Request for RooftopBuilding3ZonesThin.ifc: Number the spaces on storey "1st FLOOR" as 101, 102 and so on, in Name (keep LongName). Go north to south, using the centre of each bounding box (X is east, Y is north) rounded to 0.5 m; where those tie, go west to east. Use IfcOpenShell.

First a look at what the model holds.

```python
import ifcopenshell
import ifcopenshell.util.element
import ifcopenshell.util.placement

model = ifcopenshell.open("RooftopBuilding3ZonesThin.ifc")
print(model.schema)
storey = next(s for s in model.by_type("IfcBuildingStorey") if s.Name == "1st FLOOR")
spaces = [e for e in ifcopenshell.util.element.get_decomposition(storey) if e.is_a("IfcSpace")]
for e in sorted(spaces, key=lambda e: e.id()):
    origin = ifcopenshell.util.placement.get_local_placement(e.ObjectPlacement)[:3, 3]
    print(e.id(), e.Name, e.LongName, origin.round(2) + 0.0, sep=" | ")
```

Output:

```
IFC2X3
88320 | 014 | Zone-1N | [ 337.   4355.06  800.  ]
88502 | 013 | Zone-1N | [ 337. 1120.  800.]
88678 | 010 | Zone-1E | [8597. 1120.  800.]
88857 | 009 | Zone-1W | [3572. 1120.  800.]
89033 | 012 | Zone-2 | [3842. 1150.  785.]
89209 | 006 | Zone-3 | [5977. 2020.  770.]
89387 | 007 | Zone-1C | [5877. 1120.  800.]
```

```python
import ifcopenshell
import ifcopenshell.geom
import ifcopenshell.util.element
import ifcopenshell.util.shape

model = ifcopenshell.open("RooftopBuilding3ZonesThin.ifc")
settings = ifcopenshell.geom.settings()
settings.set("use-world-coords", True)


def centre(element):
    shape = ifcopenshell.geom.create_shape(settings, element)
    return ifcopenshell.util.shape.get_bbox_centroid(shape.geometry)


storey = next(s for s in model.by_type("IfcBuildingStorey") if s.Name == "1st FLOOR")
spaces = [e for e in ifcopenshell.util.element.get_decomposition(storey) if e.is_a("IfcSpace")]

# Insertion points can sit at a corner or the storey origin, so sort by the geometry (in metres).
centres = {e: centre(e) for e in spaces}
spaces.sort(key=lambda e: (-round(centres[e][1] / 0.5), centres[e][0]))

for i, e in enumerate(spaces, start=1):
    number = f"1{i:02d}"
    e.Name = number
    print(e.id(), number)

model.write("RooftopBuilding3ZonesThin_updated.ifc")
```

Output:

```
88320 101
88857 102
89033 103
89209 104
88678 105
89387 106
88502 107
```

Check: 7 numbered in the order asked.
